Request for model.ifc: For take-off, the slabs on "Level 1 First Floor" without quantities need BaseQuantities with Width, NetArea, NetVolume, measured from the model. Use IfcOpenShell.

First a look at what the model holds.

```python
import ifcopenshell
import ifcopenshell.util.element
import ifcopenshell.util.unit

model = ifcopenshell.open("model.ifc")
print(model.schema)
for unit_type in ("LENGTHUNIT", "AREAUNIT", "VOLUMEUNIT"):
    print(unit_type, ifcopenshell.util.unit.calculate_unit_scale(model, unit_type))
storey = next(s for s in model.by_type("IfcBuildingStorey") if s.Name == "Level 1 First Floor")
slabs = [e for e in ifcopenshell.util.element.get_decomposition(storey) if e.is_a("IfcSlab")]
for e in sorted(slabs, key=lambda e: e.id()):
    print(e.id(), e.is_a(), e.Name, list(ifcopenshell.util.element.get_psets(e, qtos_only=True)), sep=" | ")
```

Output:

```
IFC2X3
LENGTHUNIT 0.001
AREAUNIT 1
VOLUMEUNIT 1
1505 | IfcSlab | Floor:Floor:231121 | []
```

```python
import ifcopenshell
import ifcopenshell.api.pset
import ifcopenshell.geom
import ifcopenshell.util.element
import ifcopenshell.util.shape
import ifcopenshell.util.unit

model = ifcopenshell.open("model.ifc")
unit_scale = ifcopenshell.util.unit.calculate_unit_scale(model)
area_scale = ifcopenshell.util.unit.calculate_unit_scale(model, "AREAUNIT")
volume_scale = ifcopenshell.util.unit.calculate_unit_scale(model, "VOLUMEUNIT")
settings = ifcopenshell.geom.settings()

storey = next(s for s in model.by_type("IfcBuildingStorey") if s.Name == "Level 1 First Floor")
slabs = [e for e in ifcopenshell.util.element.get_decomposition(storey) if e.is_a("IfcSlab")]

for e in sorted(slabs, key=lambda e: e.id()):
    if ifcopenshell.util.element.get_psets(e, qtos_only=True, should_inherit=False):
        continue
    # Geometry comes back in metres, in the element's own axes.
    shape = ifcopenshell.geom.create_shape(settings, e)
    values = {
        "Width": ifcopenshell.util.shape.get_z(shape.geometry) / unit_scale,
        "NetArea": ifcopenshell.util.shape.get_footprint_area(shape.geometry) / area_scale,
        "NetVolume": ifcopenshell.util.shape.get_volume(shape.geometry) / volume_scale,
    }
    qto = ifcopenshell.api.pset.add_qto(model, product=e, name="BaseQuantities")
    ifcopenshell.api.pset.edit_qto(model, qto=qto, properties=values)
    print(e.id(), {k: round(v, 3) for k, v in values.items()})

model.write("model_updated.ifc")
```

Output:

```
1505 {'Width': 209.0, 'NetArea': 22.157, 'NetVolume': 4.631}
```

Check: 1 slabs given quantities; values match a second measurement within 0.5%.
